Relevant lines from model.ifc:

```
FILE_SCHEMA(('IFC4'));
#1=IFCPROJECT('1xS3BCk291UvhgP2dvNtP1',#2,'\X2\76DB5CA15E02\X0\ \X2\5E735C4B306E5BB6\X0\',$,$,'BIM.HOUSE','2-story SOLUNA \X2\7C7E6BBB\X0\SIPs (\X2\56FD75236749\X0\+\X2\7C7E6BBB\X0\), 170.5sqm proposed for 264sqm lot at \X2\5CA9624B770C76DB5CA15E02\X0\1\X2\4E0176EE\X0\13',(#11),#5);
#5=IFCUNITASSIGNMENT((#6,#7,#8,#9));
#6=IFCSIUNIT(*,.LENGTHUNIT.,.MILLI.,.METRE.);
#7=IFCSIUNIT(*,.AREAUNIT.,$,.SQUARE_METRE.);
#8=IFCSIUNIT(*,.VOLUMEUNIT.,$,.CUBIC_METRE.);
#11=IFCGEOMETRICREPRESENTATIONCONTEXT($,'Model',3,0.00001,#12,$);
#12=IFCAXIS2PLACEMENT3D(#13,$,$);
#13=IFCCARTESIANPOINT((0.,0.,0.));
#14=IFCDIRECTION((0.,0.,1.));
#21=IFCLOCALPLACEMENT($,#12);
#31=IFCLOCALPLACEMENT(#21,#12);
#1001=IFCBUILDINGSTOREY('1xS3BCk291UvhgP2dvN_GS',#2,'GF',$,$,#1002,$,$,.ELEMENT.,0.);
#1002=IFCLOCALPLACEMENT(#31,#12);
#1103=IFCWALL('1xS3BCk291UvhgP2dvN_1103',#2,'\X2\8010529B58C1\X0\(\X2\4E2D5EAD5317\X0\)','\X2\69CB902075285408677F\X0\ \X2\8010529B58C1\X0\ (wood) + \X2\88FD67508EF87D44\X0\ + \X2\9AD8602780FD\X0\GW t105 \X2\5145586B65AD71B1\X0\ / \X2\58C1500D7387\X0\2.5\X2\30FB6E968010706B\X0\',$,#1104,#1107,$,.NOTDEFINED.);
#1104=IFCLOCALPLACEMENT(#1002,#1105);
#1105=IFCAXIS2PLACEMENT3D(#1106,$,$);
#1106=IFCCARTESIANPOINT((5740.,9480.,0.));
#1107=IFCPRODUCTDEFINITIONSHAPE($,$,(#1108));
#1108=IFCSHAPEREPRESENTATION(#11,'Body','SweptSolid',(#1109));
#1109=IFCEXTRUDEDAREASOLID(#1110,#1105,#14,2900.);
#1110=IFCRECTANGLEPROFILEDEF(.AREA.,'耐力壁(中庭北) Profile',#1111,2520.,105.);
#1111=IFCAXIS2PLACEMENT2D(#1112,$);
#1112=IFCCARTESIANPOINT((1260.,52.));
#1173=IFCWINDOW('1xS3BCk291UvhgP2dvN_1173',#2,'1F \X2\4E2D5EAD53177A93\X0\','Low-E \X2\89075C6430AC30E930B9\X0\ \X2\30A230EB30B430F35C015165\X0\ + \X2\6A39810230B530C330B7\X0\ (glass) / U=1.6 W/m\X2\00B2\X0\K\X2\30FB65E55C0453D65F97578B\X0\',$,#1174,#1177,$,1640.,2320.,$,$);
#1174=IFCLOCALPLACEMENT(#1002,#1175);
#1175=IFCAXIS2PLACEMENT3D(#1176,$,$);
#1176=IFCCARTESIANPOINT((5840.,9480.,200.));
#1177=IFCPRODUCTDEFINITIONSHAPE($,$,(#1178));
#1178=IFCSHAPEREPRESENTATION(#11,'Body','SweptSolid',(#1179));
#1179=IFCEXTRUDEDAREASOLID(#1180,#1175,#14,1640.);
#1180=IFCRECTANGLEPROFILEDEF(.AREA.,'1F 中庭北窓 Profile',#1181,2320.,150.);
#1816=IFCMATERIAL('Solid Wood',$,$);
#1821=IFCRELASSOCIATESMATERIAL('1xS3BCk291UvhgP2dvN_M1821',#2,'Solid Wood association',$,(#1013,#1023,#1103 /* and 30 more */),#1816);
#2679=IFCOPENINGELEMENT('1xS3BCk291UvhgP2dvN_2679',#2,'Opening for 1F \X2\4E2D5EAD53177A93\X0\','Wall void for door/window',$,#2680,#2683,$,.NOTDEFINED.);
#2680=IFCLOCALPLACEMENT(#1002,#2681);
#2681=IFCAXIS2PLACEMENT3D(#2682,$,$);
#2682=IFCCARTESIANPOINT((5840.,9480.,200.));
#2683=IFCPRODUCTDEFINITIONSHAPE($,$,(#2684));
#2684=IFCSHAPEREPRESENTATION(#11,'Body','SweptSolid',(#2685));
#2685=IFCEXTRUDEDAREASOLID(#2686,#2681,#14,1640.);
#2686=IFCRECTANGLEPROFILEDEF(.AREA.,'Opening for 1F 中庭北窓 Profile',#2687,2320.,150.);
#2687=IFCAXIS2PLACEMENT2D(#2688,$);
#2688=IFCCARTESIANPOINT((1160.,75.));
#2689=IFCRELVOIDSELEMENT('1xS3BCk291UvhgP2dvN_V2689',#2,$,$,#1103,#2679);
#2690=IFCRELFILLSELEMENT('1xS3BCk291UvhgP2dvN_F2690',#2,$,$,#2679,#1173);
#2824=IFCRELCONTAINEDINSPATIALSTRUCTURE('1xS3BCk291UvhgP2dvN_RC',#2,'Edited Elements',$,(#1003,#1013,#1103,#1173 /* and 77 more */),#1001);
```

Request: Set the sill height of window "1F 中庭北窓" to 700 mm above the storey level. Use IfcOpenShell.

```python
import numpy as np
import ifcopenshell
import ifcopenshell.api.geometry
import ifcopenshell.geom
import ifcopenshell.util.element
import ifcopenshell.util.placement
import ifcopenshell.util.shape
import ifcopenshell.util.unit

model = ifcopenshell.open("model.ifc")
unit_scale = ifcopenshell.util.unit.calculate_unit_scale(model)

window = model.by_id(1173)
opening = window.FillsVoids[0].RelatingOpeningElement
storey = ifcopenshell.util.element.get_container(window, ifc_class="IfcBuildingStorey")
level = ifcopenshell.util.placement.get_local_placement(storey.ObjectPlacement)[2, 3]

# The opening's origin need not be at the sill, so measure its lowest point.
shape = ifcopenshell.geom.create_shape(ifcopenshell.geom.settings(), opening)
bottom = ifcopenshell.util.shape.get_shape_bottom_elevation(shape, shape.geometry) / unit_scale
dz = level + 0.7 / unit_scale - bottom

shift = np.array([0.0, 0.0, dz])
# The window is not placed relative to its opening, so move both.
for product in (opening, window):
    matrix = ifcopenshell.util.placement.get_local_placement(product.ObjectPlacement)
    matrix[:3, 3] += shift
    ifcopenshell.api.geometry.edit_object_placement(model, product=product, matrix=matrix, is_si=False)

print(f"moved by {dz * unit_scale:+.3f} m")

model.write("model_updated.ifc")
```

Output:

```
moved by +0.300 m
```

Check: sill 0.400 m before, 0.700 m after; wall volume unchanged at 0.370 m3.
